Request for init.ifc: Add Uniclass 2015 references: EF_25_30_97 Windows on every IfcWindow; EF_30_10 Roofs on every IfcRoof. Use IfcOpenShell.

First a look at what the model holds.

```python
import ifcopenshell

model = ifcopenshell.open("init.ifc")
print(model.schema)
print("classifications:", [c.Name for c in model.by_type("IfcClassification")])
for ifc_class in ("IfcDoor", "IfcRoof", "IfcStair", "IfcWall", "IfcWindow"):
    print(ifc_class, len(model.by_type(ifc_class)))
```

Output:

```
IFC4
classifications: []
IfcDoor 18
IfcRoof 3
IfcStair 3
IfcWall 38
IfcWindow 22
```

```python
import ifcopenshell
import ifcopenshell.api.classification

model = ifcopenshell.open("init.ifc")

system = ifcopenshell.api.classification.add_classification(model, classification="Uniclass 2015")

codes = {
    "IfcWindow": ("EF_25_30_97", "Windows"),
    "IfcRoof": ("EF_30_10", "Roofs"),
}
for ifc_class, (code, name) in codes.items():
    products = model.by_type(ifc_class)
    ifcopenshell.api.classification.add_reference(
        model, products=products, classification=system, identification=code, name=name
    )
    print(code, len(products))

model.write("init_rev.ifc")
```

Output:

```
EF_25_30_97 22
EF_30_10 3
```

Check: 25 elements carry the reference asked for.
